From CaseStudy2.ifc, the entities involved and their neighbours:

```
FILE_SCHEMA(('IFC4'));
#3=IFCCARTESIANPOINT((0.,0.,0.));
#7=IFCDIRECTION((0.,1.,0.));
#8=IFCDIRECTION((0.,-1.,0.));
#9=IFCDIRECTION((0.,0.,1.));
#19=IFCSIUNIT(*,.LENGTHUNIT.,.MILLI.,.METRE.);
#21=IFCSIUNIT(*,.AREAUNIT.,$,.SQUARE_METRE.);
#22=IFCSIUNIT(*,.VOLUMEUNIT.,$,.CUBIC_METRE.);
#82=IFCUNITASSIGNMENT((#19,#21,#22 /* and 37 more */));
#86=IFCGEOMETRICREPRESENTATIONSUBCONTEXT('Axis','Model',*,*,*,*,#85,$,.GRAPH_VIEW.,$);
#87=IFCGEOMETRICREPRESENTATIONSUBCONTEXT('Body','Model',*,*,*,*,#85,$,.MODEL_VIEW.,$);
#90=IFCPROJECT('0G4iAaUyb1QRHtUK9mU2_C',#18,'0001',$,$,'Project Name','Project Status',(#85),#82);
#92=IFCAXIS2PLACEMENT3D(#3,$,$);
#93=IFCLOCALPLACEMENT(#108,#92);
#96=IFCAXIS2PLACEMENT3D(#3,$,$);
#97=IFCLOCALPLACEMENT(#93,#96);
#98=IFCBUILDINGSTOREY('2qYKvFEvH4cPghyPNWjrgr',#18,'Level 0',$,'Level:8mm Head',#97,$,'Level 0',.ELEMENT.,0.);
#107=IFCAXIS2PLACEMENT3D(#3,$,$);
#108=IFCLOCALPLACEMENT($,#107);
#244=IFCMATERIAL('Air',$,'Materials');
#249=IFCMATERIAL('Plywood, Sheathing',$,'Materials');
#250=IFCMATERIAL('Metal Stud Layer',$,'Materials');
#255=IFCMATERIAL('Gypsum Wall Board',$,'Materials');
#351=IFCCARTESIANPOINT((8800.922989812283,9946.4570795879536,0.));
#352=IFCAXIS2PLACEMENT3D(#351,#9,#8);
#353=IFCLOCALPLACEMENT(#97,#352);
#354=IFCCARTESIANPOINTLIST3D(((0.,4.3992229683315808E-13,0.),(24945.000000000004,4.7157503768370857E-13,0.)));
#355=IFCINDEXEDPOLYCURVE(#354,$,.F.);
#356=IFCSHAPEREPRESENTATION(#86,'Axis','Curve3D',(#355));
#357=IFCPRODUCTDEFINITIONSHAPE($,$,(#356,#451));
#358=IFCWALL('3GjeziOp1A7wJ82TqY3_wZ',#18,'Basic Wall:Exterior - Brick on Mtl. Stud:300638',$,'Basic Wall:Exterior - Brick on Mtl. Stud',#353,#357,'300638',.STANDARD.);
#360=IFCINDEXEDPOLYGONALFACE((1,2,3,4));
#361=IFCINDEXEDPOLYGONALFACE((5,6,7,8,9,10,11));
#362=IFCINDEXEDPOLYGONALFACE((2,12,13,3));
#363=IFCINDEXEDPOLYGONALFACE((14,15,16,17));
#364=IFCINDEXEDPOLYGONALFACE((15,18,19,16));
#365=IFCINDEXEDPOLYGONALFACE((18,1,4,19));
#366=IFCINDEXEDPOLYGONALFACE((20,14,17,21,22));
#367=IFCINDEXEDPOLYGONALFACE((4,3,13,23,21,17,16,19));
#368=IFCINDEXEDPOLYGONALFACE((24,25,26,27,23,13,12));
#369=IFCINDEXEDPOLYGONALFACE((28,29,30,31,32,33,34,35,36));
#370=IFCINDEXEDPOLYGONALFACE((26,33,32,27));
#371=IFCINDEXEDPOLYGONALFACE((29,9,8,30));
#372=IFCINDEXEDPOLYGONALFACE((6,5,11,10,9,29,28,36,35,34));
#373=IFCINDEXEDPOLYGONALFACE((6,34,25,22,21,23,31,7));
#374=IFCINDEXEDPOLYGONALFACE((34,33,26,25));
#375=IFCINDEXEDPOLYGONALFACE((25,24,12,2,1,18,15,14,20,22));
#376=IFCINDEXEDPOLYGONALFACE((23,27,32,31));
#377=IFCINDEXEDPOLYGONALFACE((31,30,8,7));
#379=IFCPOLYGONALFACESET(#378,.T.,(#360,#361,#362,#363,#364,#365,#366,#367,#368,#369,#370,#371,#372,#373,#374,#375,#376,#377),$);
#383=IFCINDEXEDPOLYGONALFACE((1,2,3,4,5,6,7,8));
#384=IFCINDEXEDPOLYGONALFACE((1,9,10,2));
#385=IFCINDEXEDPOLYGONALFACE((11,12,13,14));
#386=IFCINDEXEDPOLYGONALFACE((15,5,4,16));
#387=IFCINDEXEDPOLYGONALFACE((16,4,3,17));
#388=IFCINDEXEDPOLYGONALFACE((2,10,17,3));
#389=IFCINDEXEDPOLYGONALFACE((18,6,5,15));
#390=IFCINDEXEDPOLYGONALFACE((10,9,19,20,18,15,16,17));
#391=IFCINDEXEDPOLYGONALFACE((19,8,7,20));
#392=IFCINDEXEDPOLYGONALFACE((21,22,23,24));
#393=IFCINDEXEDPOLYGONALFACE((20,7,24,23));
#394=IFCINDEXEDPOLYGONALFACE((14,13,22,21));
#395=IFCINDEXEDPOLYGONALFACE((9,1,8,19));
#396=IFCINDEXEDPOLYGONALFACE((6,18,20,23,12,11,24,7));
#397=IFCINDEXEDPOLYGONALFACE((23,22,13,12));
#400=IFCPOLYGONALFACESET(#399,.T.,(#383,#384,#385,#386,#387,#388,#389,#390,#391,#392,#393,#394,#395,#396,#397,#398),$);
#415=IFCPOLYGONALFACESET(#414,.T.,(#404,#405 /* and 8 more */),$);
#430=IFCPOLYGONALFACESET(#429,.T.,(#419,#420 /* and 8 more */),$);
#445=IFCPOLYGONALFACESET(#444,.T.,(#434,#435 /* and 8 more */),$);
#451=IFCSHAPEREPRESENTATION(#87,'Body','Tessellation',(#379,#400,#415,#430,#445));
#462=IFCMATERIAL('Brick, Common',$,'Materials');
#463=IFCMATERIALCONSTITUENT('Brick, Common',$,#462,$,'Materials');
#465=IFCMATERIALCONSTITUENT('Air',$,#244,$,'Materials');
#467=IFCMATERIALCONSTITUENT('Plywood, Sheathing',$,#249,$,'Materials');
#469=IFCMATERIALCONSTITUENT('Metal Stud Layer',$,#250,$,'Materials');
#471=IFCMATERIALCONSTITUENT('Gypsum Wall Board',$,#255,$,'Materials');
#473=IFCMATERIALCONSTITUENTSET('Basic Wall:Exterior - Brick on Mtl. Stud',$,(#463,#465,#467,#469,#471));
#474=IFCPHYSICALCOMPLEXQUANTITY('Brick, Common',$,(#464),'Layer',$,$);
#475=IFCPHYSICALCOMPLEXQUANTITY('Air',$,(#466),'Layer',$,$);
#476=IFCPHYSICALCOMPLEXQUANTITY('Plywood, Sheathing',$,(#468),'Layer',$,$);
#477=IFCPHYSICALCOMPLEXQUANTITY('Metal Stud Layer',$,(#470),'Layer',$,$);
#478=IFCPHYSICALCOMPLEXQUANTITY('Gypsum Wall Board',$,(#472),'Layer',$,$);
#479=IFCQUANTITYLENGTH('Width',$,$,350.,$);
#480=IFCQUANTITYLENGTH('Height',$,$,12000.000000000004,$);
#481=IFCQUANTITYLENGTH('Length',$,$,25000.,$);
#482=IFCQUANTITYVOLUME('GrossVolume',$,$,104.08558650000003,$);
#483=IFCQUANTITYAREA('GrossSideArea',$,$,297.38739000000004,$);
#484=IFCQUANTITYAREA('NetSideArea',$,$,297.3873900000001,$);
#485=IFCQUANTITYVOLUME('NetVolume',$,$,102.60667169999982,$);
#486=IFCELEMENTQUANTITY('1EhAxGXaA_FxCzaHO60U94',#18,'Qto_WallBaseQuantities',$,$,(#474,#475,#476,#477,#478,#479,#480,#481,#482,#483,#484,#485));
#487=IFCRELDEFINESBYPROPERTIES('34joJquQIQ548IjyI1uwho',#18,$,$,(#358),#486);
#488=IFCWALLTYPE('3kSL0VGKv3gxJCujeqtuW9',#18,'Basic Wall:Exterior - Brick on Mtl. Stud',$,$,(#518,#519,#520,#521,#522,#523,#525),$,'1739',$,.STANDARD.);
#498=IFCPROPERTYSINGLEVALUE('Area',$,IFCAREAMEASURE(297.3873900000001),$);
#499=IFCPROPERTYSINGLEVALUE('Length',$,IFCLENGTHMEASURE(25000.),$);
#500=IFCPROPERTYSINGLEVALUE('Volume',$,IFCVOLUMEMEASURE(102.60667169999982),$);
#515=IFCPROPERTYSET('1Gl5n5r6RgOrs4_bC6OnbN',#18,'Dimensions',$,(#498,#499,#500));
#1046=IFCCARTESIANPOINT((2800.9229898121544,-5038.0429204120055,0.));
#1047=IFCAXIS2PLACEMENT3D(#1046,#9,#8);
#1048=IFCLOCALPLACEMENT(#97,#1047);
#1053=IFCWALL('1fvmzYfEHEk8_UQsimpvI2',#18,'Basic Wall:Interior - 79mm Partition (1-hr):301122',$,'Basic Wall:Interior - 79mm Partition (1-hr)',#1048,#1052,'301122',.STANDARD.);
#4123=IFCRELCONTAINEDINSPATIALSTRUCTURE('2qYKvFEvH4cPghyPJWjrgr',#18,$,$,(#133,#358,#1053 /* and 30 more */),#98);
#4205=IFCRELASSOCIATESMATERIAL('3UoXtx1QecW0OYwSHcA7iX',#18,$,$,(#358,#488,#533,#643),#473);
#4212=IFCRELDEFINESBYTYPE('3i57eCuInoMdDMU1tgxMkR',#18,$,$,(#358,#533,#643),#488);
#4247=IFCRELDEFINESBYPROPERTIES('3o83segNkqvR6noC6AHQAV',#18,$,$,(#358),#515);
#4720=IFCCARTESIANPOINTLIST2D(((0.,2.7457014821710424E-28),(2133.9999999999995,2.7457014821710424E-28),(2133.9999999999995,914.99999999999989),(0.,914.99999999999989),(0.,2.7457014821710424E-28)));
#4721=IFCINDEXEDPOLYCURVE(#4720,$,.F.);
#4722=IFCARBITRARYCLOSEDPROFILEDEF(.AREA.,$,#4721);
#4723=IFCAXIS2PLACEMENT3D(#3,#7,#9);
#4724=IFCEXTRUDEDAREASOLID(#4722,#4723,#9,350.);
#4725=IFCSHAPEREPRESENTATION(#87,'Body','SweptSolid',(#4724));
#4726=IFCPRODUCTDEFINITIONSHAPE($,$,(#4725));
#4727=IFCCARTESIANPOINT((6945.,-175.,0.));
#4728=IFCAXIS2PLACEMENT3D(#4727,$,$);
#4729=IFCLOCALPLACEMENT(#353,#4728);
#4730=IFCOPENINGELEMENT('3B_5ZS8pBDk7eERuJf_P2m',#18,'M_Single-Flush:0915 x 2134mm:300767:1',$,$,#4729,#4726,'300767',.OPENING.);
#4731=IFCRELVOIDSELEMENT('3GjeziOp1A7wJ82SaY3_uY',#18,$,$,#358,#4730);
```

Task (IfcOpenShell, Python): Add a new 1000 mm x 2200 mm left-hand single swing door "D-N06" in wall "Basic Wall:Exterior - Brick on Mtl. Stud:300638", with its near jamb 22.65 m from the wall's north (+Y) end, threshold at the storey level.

```python
import numpy as np
import ifcopenshell
import ifcopenshell.api.feature
import ifcopenshell.api.geometry
import ifcopenshell.api.pset
import ifcopenshell.api.root
import ifcopenshell.api.spatial
import ifcopenshell.geom
import ifcopenshell.util.element
import ifcopenshell.util.placement
import ifcopenshell.util.representation
import ifcopenshell.util.shape
import ifcopenshell.util.unit

model = ifcopenshell.open("CaseStudy2.ifc")
unit_scale = ifcopenshell.util.unit.calculate_unit_scale(model)
area_scale = ifcopenshell.util.unit.calculate_unit_scale(model, "AREAUNIT")
volume_scale = ifcopenshell.util.unit.calculate_unit_scale(model, "VOLUMEUNIT")
settings = ifcopenshell.geom.settings()


def volume(element):
    """Net volume in cubic metres, openings subtracted."""
    shape = ifcopenshell.geom.create_shape(settings, element)
    return ifcopenshell.util.shape.get_volume(shape.geometry)


wall = model.by_guid("3GjeziOp1A7wJ82TqY3_wZ")
storey = ifcopenshell.util.element.get_container(wall, ifc_class="IfcBuildingStorey")
context = ifcopenshell.util.representation.get_context(model, "Model", "Body", "MODEL_VIEW")
before = volume(wall)

width, height, from_end, sill = 1, 2.2, 22.65, 0.0  # metres

# The wall runs along its own X axis, and the end named is its -X end.
wall_shape = ifcopenshell.geom.create_shape(settings, wall)
x, y, z = ifcopenshell.util.shape.get_vertices(wall_shape.geometry).T
start = x.min() + from_end
face, thickness = float(y.min()), float(y.max() - y.min())
wall_matrix = ifcopenshell.util.placement.get_local_placement(wall.ObjectPlacement)
level = ifcopenshell.util.placement.get_local_placement(storey.ObjectPlacement)[2, 3]


def in_wall(x, y):
    """Placement at x, y metres in the wall's axes, at sill height."""
    matrix = wall_matrix.copy()
    matrix[:, 3] = wall_matrix @ np.array([x / unit_scale, y / unit_scale, 0.0, 1.0])
    matrix[2, 3] = level + sill / unit_scale
    return matrix


# Opening: a box that overshoots both wall faces by 50 mm.
opening = ifcopenshell.api.root.create_entity(model, ifc_class="IfcOpeningElement", predefined_type="OPENING")
box = ifcopenshell.api.geometry.add_wall_representation(
    model, context=context, length=width, height=height, thickness=thickness + 0.1
)
ifcopenshell.api.geometry.assign_representation(model, product=opening, representation=box)
ifcopenshell.api.geometry.edit_object_placement(model, product=opening, matrix=in_wall(start, face - 0.05), is_si=False)
ifcopenshell.api.feature.add_feature(model, feature=opening, element=wall)

door = ifcopenshell.api.root.create_entity(model, ifc_class="IfcDoor", name="D-N06", predefined_type="DOOR")
door.OverallWidth, door.OverallHeight = width / unit_scale, height / unit_scale
door.OperationType = "SINGLE_SWING_LEFT"
body = ifcopenshell.api.geometry.add_door_representation(
    model,
    context=context,
    overall_width=door.OverallWidth,
    overall_height=door.OverallHeight,
    operation_type="SINGLE_SWING_LEFT",
    lining_properties={"LiningDepth": thickness / unit_scale, "ThresholdDepth": thickness / unit_scale},
)
ifcopenshell.api.geometry.assign_representation(model, product=door, representation=body)
ifcopenshell.api.spatial.assign_container(model, products=[door], relating_structure=storey)
ifcopenshell.api.feature.add_filling(model, opening=opening, element=door)

# The lining spans the wall, so the door starts at the wall face.
ifcopenshell.api.geometry.edit_object_placement(model, product=door, matrix=in_wall(start, face), is_si=False)

after = volume(wall)

# Update the wall's stored quantities.
qto = model.by_id(ifcopenshell.util.element.get_pset(wall, "Qto_WallBaseQuantities", should_inherit=False)["id"])
ifcopenshell.api.pset.edit_qto(model, qto=qto, properties={
    "NetSideArea": after / thickness / area_scale,
    "NetVolume": after / volume_scale,
})
pset = model.by_id(ifcopenshell.util.element.get_pset(wall, "Dimensions", should_inherit=False)["id"])
ifcopenshell.api.pset.edit_pset(model, pset=pset, properties={
    "Area": model.create_entity("IfcAreaMeasure", after / thickness / area_scale),
    "Volume": model.create_entity("IfcVolumeMeasure", after / volume_scale),
})

print(f"wall volume {before:.3f} -> {after:.3f} m3")

model.write("CaseStudy2-out.ifc")
```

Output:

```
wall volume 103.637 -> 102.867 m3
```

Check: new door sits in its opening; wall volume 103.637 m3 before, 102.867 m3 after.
